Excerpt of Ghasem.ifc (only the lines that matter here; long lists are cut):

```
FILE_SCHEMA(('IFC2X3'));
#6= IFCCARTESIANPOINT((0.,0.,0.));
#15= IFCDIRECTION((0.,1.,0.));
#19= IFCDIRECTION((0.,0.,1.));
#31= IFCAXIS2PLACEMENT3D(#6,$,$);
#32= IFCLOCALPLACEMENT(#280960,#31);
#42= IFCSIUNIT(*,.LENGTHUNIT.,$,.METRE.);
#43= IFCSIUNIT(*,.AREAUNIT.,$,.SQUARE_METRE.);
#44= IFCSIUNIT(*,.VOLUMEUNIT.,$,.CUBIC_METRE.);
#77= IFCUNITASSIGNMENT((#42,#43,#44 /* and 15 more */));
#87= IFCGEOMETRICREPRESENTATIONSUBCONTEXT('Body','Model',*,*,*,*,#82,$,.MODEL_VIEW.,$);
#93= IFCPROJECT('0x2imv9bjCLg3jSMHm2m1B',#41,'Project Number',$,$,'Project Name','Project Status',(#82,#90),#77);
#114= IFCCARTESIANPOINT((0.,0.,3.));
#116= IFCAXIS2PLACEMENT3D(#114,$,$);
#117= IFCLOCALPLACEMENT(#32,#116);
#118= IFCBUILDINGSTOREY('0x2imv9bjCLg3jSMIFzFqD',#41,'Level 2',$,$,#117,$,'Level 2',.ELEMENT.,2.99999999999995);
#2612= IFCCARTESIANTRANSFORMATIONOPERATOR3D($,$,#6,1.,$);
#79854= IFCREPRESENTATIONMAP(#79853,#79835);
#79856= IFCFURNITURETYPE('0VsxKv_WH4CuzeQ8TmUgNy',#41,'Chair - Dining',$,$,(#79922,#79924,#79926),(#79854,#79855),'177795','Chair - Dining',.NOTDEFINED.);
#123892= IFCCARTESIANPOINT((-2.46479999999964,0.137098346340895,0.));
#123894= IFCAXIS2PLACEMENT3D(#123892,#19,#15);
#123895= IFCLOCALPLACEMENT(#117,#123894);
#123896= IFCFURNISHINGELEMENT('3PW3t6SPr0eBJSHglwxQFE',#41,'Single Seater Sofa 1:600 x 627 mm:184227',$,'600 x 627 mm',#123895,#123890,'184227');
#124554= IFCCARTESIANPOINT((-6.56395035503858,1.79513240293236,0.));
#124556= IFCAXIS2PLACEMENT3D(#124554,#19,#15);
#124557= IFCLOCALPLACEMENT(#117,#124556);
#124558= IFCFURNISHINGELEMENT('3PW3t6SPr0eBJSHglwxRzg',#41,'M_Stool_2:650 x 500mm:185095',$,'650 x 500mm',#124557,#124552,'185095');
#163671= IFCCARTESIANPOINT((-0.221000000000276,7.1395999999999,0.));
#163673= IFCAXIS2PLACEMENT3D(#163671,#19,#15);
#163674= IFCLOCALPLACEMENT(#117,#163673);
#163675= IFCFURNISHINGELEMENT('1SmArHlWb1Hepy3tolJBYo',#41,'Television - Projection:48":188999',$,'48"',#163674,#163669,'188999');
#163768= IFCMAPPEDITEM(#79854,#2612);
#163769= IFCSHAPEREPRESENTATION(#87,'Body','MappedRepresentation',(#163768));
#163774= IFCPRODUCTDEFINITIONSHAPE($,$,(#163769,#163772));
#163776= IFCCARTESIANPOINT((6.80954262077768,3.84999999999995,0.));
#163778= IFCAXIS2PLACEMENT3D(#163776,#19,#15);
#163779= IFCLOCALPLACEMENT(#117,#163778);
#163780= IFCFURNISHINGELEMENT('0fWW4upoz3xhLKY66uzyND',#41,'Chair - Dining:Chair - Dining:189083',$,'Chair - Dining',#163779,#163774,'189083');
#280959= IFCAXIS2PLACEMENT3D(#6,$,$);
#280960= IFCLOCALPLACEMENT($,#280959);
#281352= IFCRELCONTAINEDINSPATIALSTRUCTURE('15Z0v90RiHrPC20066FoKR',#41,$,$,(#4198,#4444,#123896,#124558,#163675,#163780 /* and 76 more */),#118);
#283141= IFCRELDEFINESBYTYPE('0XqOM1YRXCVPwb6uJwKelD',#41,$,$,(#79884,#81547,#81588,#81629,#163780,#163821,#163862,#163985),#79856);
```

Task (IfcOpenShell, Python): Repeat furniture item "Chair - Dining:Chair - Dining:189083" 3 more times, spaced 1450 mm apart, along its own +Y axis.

```python
import ifcopenshell
import ifcopenshell.api.geometry
import ifcopenshell.api.root
import ifcopenshell.util.element
import ifcopenshell.util.placement
import ifcopenshell.util.unit

model = ifcopenshell.open("Ghasem.ifc")
unit_scale = ifcopenshell.util.unit.calculate_unit_scale(model)


def reuse_history(source, copy):
    """copy_class also copies each property set's owner history, people and application; keep the originals."""
    for rel in copy.IsDefinedBy:
        if rel.is_a("IfcRelDefinesByProperties") and (history := rel.RelatingPropertyDefinition.OwnerHistory):
            rel.RelatingPropertyDefinition.OwnerHistory = source.OwnerHistory
            ifcopenshell.util.element.remove_deep2(model, history)


source = model.by_id(163780)
base = ifcopenshell.util.placement.get_local_placement(source.ObjectPlacement)
step = base[:3, 1] * 1.45 / unit_scale

for i in range(1, 4):
    copy = ifcopenshell.api.root.copy_class(model, product=source)
    copy.Representation = ifcopenshell.util.element.copy_deep(
        model, source.Representation, exclude=["IfcGeometricRepresentationContext", "IfcRepresentationMap"]
    )
    copy.Name = "Chair - Dining:Chair - Dining"
    copy.Tag = None
    reuse_history(source, copy)
    matrix = base.copy()
    matrix[:3, 3] += i * step
    print("added at", matrix[:3, 3].round(3) + 0.0)
    ifcopenshell.api.geometry.edit_object_placement(model, product=copy, matrix=matrix, is_si=False)

model.write("Ghasem_rev.ifc")
```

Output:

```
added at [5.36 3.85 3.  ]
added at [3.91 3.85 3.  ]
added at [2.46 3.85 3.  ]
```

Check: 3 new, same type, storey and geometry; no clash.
